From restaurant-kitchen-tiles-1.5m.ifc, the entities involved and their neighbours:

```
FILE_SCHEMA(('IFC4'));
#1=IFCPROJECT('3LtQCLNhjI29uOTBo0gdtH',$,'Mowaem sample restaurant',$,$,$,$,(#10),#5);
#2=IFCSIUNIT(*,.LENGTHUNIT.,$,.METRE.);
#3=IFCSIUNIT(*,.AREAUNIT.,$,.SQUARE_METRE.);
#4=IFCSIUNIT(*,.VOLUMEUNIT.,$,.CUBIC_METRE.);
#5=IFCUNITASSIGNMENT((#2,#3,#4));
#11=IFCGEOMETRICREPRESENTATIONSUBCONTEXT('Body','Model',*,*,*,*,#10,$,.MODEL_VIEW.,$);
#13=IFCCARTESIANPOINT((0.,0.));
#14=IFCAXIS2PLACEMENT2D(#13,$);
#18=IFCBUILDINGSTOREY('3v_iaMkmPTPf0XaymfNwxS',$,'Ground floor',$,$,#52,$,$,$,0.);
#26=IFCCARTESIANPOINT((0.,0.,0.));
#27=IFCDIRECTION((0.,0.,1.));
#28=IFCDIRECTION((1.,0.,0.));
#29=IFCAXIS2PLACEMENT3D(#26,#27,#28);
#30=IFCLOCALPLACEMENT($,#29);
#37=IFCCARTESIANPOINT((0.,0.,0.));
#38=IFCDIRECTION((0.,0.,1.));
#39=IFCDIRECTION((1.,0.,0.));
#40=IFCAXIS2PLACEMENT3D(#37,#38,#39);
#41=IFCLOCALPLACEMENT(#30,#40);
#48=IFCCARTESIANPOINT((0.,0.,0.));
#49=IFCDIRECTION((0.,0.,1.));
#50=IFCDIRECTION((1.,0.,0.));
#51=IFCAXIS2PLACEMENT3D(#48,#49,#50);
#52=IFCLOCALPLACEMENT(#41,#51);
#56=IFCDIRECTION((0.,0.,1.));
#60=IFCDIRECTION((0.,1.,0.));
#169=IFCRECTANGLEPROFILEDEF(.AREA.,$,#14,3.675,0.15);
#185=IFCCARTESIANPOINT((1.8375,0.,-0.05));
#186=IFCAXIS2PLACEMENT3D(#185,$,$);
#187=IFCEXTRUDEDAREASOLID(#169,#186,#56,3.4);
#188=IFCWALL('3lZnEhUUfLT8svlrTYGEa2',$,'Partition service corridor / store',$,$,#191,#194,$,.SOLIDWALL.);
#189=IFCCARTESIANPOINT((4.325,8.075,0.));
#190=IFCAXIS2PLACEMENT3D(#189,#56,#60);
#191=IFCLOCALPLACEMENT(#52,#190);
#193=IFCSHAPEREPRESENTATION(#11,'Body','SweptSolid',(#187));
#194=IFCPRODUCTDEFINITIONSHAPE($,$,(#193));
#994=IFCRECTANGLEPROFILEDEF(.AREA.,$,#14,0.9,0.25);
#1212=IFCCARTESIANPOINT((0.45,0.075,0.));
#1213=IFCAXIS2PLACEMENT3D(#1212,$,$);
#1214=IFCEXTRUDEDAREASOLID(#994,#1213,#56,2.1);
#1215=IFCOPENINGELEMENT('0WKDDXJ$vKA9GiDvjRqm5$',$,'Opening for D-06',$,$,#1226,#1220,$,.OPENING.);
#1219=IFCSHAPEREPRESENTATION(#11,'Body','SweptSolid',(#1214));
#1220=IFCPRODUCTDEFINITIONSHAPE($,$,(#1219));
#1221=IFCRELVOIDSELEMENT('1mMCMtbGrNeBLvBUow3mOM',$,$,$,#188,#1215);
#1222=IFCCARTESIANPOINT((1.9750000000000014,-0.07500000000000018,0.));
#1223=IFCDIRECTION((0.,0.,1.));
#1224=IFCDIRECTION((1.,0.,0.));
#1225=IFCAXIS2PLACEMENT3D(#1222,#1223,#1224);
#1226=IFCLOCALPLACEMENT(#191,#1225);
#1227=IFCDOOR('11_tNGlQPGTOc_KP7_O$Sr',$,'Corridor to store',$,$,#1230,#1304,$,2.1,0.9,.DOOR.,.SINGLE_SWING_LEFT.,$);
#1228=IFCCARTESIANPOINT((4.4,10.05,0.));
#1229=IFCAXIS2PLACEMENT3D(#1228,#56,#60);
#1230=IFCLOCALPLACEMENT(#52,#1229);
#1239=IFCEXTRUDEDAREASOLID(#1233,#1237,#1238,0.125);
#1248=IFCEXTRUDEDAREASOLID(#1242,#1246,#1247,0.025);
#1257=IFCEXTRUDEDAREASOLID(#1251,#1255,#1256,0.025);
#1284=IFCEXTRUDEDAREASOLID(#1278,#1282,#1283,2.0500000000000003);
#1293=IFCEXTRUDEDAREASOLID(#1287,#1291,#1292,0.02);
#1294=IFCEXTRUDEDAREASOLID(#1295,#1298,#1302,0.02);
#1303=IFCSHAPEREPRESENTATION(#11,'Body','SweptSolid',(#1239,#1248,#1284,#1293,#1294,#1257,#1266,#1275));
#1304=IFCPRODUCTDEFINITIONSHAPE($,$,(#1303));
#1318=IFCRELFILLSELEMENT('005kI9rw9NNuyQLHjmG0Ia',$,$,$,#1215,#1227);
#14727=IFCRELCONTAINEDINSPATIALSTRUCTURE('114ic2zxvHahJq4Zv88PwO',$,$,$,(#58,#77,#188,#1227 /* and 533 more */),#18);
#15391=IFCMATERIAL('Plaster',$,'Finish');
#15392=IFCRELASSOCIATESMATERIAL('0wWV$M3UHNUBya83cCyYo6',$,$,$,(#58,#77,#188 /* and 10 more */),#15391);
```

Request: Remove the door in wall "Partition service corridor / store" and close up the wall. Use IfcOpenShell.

```python
import ifcopenshell
import ifcopenshell.api.feature
import ifcopenshell.api.root
import ifcopenshell.geom
import ifcopenshell.util.shape

model = ifcopenshell.open("restaurant-kitchen-tiles-1.5m.ifc")
settings = ifcopenshell.geom.settings()


def volume(element):
    """Net volume in cubic metres, openings subtracted."""
    shape = ifcopenshell.geom.create_shape(settings, element)
    return ifcopenshell.util.shape.get_volume(shape.geometry)


door = model.by_id(1227)
opening = door.FillsVoids[0].RelatingOpeningElement
wall = opening.VoidsElements[0].RelatingBuildingElement
before = volume(wall)

ifcopenshell.api.root.remove_product(model, product=door)
ifcopenshell.api.feature.remove_feature(model, feature=opening)

after = volume(wall)

print(f"wall volume {before:.3f} -> {after:.3f} m3")

model.write("restaurant-kitchen-tiles-1.5m_v2.ifc")
```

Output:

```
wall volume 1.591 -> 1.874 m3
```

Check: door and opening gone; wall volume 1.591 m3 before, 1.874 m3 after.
